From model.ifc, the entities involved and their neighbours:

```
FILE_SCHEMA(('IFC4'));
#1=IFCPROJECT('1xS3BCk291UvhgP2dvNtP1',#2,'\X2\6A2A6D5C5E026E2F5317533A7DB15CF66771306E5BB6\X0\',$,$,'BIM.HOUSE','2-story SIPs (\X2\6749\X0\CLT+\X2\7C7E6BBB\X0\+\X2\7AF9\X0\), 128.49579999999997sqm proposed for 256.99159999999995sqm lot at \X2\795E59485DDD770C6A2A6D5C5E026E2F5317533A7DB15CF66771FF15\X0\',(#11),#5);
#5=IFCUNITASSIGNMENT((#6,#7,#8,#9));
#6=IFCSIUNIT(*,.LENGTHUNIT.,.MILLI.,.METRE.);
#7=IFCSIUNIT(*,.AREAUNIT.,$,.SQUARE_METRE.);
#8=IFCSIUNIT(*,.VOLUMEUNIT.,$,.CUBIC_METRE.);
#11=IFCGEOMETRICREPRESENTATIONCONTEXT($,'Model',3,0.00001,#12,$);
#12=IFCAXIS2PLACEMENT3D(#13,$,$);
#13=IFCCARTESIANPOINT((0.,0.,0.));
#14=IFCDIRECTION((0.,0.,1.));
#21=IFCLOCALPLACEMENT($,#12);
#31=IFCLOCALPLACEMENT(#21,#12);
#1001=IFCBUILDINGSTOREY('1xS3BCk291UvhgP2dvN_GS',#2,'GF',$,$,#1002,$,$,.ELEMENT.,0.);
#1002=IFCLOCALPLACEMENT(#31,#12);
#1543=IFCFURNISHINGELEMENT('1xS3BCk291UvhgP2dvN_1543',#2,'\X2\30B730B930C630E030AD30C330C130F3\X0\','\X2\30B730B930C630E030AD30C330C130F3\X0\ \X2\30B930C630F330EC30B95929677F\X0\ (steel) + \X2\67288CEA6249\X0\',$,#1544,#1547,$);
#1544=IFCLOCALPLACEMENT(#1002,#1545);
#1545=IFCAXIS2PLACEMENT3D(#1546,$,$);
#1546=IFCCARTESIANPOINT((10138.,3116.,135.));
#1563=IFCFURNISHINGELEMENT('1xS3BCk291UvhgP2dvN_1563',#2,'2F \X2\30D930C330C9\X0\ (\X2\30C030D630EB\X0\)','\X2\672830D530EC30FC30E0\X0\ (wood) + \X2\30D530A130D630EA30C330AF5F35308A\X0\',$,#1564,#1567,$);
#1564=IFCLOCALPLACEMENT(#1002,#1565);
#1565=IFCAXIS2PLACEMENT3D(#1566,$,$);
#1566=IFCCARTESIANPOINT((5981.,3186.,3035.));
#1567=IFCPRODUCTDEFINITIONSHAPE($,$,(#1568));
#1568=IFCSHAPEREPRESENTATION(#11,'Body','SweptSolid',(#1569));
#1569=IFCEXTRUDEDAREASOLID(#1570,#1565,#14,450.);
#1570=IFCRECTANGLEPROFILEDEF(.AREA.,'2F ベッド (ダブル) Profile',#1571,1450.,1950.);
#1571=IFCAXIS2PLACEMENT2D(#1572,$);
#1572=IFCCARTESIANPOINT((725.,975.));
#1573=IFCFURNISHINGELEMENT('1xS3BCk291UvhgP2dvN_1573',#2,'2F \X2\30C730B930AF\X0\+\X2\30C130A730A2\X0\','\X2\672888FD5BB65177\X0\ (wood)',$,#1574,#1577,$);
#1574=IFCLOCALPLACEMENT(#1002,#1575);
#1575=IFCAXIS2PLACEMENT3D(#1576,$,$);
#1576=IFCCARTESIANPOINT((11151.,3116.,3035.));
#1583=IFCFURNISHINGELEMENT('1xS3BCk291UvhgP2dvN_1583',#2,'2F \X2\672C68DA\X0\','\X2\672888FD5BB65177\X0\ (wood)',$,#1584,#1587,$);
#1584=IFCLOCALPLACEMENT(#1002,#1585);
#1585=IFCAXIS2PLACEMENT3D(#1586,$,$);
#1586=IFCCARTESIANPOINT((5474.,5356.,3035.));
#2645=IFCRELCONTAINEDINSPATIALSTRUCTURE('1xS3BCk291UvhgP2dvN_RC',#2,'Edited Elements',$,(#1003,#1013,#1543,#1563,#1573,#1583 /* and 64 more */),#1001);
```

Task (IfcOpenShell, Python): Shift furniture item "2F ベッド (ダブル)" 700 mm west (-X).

```python
import ifcopenshell
import ifcopenshell.api.geometry
import ifcopenshell.util.placement
import ifcopenshell.util.unit

model = ifcopenshell.open("model.ifc")
unit_scale = ifcopenshell.util.unit.calculate_unit_scale(model)

item = model.by_guid("1xS3BCk291UvhgP2dvN_1563")
matrix = ifcopenshell.util.placement.get_local_placement(item.ObjectPlacement)
matrix[0, 3] -= 0.7 / unit_scale
ifcopenshell.api.geometry.edit_object_placement(model, product=item, matrix=matrix, is_si=False)

print(ifcopenshell.util.placement.get_local_placement(item.ObjectPlacement).round(3) + 0.0)

model.write("model-out.ifc")
```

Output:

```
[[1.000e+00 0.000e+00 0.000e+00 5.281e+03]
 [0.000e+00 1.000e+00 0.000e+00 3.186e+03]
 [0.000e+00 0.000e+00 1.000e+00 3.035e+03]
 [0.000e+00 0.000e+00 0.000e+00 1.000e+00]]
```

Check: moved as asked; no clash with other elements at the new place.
